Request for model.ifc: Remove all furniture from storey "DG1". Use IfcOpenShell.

First a look at what the model holds.

```python
import ifcopenshell
import ifcopenshell.util.element

model = ifcopenshell.open("model.ifc")
print(model.schema)
storey = next(s for s in model.by_type("IfcBuildingStorey") if s.Name == "DG1")
furniture = [e for e in ifcopenshell.util.element.get_decomposition(storey) if e.is_a("IfcFurnishingElement")]
seen = {}
for e in furniture:
    element_type = ifcopenshell.util.element.get_type(e)
    name = element_type.Name if element_type not in (None, e) else None
    seen[name] = seen.get(name, 0) + 1
for name, count in sorted(seen.items(), key=str):
    print(count, "x", name)
```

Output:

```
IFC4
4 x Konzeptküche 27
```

```python
import ifcopenshell
import ifcopenshell.api.root
import ifcopenshell.util.element

model = ifcopenshell.open("model.ifc")

storey = next(s for s in model.by_type("IfcBuildingStorey") if s.Name == "DG1")
furniture = [e for e in ifcopenshell.util.element.get_decomposition(storey) if e.is_a("IfcFurnishingElement")]

for e in furniture:
    ifcopenshell.api.root.remove_product(model, product=e)
print(len(furniture), "removed")

model.write("model_v2.ifc")
```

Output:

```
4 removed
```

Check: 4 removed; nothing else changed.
